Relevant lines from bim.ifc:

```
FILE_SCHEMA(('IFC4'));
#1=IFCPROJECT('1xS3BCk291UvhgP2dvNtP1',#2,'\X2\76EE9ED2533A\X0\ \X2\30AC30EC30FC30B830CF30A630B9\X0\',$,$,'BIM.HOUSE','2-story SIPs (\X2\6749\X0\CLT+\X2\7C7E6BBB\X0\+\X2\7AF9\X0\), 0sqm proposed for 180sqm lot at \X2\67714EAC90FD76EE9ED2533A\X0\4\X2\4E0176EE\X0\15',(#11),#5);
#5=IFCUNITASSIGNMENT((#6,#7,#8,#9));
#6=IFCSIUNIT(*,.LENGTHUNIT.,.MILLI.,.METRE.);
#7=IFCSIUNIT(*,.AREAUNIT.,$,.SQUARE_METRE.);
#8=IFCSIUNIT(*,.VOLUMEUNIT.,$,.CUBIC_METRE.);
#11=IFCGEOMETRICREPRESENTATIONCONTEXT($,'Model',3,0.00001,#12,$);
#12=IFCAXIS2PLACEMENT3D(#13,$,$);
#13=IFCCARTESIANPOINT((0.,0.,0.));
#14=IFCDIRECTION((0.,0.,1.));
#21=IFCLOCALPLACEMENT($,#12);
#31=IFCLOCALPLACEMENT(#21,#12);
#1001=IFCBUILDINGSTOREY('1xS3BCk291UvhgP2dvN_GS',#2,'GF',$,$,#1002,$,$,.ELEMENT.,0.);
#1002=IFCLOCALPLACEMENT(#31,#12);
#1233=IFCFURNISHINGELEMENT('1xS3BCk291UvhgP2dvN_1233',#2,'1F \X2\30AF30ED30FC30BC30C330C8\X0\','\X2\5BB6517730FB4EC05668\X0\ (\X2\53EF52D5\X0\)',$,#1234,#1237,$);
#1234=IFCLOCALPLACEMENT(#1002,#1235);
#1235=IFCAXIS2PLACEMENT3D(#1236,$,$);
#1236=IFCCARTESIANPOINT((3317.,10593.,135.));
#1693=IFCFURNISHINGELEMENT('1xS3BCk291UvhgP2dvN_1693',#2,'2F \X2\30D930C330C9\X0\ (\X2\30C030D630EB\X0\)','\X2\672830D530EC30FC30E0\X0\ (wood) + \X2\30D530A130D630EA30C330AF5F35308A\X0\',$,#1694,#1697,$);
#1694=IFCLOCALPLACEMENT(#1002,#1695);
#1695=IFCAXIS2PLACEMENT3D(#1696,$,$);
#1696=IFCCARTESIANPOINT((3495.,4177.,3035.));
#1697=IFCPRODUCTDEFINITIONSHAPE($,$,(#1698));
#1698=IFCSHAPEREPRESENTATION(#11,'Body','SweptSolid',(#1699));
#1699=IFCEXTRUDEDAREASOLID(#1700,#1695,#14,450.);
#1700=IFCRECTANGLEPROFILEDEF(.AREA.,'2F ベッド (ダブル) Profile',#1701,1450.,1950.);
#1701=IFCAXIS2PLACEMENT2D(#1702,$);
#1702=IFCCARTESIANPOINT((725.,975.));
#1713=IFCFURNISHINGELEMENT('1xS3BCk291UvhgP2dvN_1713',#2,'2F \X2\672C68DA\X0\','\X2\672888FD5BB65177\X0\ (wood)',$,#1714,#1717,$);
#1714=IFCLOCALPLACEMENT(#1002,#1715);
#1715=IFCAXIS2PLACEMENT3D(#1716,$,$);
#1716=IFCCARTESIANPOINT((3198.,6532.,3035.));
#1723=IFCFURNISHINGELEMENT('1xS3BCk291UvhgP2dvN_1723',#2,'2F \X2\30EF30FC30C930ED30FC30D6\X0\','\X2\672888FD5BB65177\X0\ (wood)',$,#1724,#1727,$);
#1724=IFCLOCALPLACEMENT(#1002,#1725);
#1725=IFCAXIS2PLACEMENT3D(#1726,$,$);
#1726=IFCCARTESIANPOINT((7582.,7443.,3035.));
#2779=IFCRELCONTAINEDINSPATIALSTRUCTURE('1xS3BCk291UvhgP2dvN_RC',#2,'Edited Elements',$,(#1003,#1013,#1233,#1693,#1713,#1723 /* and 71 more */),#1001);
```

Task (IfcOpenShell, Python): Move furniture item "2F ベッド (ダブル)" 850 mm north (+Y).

```python
import ifcopenshell
import ifcopenshell.api.geometry
import ifcopenshell.util.placement

model = ifcopenshell.open("bim.ifc")

item = model.by_guid("1xS3BCk291UvhgP2dvN_1693")
matrix = ifcopenshell.util.placement.get_local_placement(item.ObjectPlacement)
matrix[1, 3] += 850.0
ifcopenshell.api.geometry.edit_object_placement(model, product=item, matrix=matrix, is_si=False)

print(ifcopenshell.util.placement.get_local_placement(item.ObjectPlacement).round(3) + 0.0)

model.write("bim_updated.ifc")
```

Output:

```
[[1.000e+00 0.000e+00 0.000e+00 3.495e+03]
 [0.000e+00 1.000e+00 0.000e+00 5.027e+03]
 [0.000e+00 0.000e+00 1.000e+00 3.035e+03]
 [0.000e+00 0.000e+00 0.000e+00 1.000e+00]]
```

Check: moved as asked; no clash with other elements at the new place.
